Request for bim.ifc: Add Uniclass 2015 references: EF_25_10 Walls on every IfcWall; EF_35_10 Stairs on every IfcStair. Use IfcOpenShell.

First a look at what the model holds.

```python
import ifcopenshell

model = ifcopenshell.open("bim.ifc")
print(model.schema)
print("classifications:", [c.Name for c in model.by_type("IfcClassification")])
for ifc_class in ("IfcDoor", "IfcRoof", "IfcStair", "IfcWall", "IfcWindow"):
    print(ifc_class, len(model.by_type(ifc_class)))
```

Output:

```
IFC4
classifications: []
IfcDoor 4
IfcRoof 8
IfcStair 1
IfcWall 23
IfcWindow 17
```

```python
import ifcopenshell
import ifcopenshell.api.classification

model = ifcopenshell.open("bim.ifc")

system = ifcopenshell.api.classification.add_classification(model, classification="Uniclass 2015")

codes = {
    "IfcWall": ("EF_25_10", "Walls"),
    "IfcStair": ("EF_35_10", "Stairs"),
}
for ifc_class, (code, name) in codes.items():
    products = model.by_type(ifc_class)
    ifcopenshell.api.classification.add_reference(
        model, products=products, classification=system, identification=code, name=name
    )
    print(code, len(products))

model.write("bim_edited.ifc")
```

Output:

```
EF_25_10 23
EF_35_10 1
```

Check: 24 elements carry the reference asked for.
